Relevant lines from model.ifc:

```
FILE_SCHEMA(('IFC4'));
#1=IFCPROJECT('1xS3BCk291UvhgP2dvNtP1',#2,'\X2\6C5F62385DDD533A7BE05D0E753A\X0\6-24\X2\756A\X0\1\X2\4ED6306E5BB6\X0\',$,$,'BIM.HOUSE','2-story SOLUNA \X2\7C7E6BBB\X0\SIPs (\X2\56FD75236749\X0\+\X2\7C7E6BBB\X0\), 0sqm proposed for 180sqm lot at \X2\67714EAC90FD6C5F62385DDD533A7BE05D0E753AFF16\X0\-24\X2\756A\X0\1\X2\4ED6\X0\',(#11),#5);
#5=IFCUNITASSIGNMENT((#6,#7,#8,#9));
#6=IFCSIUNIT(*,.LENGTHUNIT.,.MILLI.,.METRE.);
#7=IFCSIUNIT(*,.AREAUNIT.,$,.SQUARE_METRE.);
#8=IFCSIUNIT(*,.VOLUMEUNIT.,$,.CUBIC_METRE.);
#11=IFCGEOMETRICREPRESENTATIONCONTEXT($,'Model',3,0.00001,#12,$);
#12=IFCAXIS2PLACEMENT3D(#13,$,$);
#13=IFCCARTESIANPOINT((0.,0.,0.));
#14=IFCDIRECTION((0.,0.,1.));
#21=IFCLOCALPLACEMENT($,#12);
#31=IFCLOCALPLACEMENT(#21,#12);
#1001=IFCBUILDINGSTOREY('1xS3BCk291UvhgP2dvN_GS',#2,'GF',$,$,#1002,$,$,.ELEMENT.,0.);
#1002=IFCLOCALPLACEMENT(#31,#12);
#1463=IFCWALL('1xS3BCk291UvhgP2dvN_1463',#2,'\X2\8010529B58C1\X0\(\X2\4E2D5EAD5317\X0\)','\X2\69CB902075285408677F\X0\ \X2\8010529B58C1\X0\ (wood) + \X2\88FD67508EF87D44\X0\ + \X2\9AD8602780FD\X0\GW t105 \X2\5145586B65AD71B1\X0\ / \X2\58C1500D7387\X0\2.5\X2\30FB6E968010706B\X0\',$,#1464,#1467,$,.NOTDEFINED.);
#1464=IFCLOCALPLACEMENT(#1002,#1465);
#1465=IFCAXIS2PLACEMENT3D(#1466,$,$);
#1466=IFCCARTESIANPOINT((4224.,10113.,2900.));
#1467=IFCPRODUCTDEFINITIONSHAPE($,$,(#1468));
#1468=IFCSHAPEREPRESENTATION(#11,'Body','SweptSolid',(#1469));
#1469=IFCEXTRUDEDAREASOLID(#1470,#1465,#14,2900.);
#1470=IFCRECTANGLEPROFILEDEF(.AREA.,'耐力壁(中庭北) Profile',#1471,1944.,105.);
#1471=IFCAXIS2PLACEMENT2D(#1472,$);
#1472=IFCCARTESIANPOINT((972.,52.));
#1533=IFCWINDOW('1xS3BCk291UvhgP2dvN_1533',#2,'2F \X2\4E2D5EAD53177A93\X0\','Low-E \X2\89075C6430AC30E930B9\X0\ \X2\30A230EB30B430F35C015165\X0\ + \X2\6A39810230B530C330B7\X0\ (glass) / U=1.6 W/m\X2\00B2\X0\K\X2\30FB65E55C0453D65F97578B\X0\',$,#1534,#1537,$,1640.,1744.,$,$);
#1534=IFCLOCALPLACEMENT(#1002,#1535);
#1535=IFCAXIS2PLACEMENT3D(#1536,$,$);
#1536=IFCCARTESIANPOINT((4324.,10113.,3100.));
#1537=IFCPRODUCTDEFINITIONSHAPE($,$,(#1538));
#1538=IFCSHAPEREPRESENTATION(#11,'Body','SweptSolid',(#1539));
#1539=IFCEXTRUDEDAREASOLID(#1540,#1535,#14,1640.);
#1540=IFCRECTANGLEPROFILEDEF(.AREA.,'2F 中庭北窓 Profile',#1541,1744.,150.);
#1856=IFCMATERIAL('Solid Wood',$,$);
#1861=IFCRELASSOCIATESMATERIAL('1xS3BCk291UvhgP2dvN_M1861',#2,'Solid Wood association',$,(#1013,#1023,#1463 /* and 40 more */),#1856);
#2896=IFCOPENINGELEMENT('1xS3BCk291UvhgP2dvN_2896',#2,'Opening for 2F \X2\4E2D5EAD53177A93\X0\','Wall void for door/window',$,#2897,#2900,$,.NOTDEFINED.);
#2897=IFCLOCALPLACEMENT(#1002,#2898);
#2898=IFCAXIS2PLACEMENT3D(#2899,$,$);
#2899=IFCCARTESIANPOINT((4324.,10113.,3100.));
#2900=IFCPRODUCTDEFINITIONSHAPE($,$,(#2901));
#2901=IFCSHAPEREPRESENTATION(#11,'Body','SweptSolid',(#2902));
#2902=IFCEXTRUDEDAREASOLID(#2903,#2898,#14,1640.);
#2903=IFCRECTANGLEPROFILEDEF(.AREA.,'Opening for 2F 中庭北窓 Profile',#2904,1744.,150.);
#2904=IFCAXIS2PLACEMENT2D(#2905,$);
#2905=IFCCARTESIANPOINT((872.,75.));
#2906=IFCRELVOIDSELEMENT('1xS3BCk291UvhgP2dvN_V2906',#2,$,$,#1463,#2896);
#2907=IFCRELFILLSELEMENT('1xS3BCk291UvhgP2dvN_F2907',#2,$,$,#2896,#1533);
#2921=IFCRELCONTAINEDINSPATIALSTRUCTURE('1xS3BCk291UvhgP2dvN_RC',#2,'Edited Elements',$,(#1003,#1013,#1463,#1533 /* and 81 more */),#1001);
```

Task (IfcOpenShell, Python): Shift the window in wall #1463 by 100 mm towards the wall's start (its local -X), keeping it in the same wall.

```python
import ifcopenshell
import ifcopenshell.api.geometry
import ifcopenshell.util.placement
import ifcopenshell.util.unit

model = ifcopenshell.open("model.ifc")
unit_scale = ifcopenshell.util.unit.calculate_unit_scale(model)

window = model.by_id(1533)
opening = window.FillsVoids[0].RelatingOpeningElement
wall = opening.VoidsElements[0].RelatingBuildingElement

wall_matrix = ifcopenshell.util.placement.get_local_placement(wall.ObjectPlacement)
shift = wall_matrix[:3, 0] * -0.1 / unit_scale
before = ifcopenshell.util.placement.get_local_placement(window.ObjectPlacement)[:3, 3].copy()

# The window is not placed relative to its opening, so move both.
for product in (opening, window):
    matrix = ifcopenshell.util.placement.get_local_placement(product.ObjectPlacement)
    matrix[:3, 3] += shift
    ifcopenshell.api.geometry.edit_object_placement(model, product=product, matrix=matrix, is_si=False)

after = ifcopenshell.util.placement.get_local_placement(window.ObjectPlacement)[:3, 3]
print("window moved by", (after - before).round(3) + 0.0)

model.write("model-out.ifc")
```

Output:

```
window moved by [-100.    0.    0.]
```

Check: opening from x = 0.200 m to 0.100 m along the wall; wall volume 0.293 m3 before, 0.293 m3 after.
